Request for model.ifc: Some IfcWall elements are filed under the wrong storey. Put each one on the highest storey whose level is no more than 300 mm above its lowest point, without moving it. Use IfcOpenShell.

First a look at what the model holds.

```python
import ifcopenshell
import ifcopenshell.util.element
import ifcopenshell.util.placement

model = ifcopenshell.open("model.ifc")
print(model.schema)
for storey in model.by_type("IfcBuildingStorey"):
    level = ifcopenshell.util.placement.get_storey_elevation(storey)
    count = sum(e.is_a("IfcWall") for e in ifcopenshell.util.element.get_contained(storey))
    print(storey.id(), storey.Name, round(level, 3), count, sep=" | ")
```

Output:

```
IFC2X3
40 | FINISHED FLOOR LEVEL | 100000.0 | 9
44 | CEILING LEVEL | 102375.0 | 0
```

```python
import ifcopenshell
import ifcopenshell.api.spatial
import ifcopenshell.geom
import ifcopenshell.util.element
import ifcopenshell.util.placement
import ifcopenshell.util.shape
import ifcopenshell.util.unit

model = ifcopenshell.open("model.ifc")
unit_scale = ifcopenshell.util.unit.calculate_unit_scale(model)
settings = ifcopenshell.geom.settings()

levels = sorted(
    ((ifcopenshell.util.placement.get_storey_elevation(s) * unit_scale, s) for s in model.by_type("IfcBuildingStorey")),
    key=lambda pair: pair[0],
)

for e in model.by_type("IfcWall"):
    current = e.ContainedInStructure[0].RelatingStructure if e.ContainedInStructure else None
    if current is None or not current.is_a("IfcBuildingStorey"):
        continue
    shape = ifcopenshell.geom.create_shape(settings, e)
    bottom = ifcopenshell.util.shape.get_shape_bottom_elevation(shape, shape.geometry)
    below = [s for level, s in levels if level <= bottom + 0.3]
    storey = below[-1] if below else levels[0][1]
    if storey != current:
        # assign_container keeps the world position.
        ifcopenshell.api.spatial.assign_container(model, products=[e], relating_structure=storey)
        print(e.id(), current.Name, "->", storey.Name)

model.write("model_updated.ifc")
```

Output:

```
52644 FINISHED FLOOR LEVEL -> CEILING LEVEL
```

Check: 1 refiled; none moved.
